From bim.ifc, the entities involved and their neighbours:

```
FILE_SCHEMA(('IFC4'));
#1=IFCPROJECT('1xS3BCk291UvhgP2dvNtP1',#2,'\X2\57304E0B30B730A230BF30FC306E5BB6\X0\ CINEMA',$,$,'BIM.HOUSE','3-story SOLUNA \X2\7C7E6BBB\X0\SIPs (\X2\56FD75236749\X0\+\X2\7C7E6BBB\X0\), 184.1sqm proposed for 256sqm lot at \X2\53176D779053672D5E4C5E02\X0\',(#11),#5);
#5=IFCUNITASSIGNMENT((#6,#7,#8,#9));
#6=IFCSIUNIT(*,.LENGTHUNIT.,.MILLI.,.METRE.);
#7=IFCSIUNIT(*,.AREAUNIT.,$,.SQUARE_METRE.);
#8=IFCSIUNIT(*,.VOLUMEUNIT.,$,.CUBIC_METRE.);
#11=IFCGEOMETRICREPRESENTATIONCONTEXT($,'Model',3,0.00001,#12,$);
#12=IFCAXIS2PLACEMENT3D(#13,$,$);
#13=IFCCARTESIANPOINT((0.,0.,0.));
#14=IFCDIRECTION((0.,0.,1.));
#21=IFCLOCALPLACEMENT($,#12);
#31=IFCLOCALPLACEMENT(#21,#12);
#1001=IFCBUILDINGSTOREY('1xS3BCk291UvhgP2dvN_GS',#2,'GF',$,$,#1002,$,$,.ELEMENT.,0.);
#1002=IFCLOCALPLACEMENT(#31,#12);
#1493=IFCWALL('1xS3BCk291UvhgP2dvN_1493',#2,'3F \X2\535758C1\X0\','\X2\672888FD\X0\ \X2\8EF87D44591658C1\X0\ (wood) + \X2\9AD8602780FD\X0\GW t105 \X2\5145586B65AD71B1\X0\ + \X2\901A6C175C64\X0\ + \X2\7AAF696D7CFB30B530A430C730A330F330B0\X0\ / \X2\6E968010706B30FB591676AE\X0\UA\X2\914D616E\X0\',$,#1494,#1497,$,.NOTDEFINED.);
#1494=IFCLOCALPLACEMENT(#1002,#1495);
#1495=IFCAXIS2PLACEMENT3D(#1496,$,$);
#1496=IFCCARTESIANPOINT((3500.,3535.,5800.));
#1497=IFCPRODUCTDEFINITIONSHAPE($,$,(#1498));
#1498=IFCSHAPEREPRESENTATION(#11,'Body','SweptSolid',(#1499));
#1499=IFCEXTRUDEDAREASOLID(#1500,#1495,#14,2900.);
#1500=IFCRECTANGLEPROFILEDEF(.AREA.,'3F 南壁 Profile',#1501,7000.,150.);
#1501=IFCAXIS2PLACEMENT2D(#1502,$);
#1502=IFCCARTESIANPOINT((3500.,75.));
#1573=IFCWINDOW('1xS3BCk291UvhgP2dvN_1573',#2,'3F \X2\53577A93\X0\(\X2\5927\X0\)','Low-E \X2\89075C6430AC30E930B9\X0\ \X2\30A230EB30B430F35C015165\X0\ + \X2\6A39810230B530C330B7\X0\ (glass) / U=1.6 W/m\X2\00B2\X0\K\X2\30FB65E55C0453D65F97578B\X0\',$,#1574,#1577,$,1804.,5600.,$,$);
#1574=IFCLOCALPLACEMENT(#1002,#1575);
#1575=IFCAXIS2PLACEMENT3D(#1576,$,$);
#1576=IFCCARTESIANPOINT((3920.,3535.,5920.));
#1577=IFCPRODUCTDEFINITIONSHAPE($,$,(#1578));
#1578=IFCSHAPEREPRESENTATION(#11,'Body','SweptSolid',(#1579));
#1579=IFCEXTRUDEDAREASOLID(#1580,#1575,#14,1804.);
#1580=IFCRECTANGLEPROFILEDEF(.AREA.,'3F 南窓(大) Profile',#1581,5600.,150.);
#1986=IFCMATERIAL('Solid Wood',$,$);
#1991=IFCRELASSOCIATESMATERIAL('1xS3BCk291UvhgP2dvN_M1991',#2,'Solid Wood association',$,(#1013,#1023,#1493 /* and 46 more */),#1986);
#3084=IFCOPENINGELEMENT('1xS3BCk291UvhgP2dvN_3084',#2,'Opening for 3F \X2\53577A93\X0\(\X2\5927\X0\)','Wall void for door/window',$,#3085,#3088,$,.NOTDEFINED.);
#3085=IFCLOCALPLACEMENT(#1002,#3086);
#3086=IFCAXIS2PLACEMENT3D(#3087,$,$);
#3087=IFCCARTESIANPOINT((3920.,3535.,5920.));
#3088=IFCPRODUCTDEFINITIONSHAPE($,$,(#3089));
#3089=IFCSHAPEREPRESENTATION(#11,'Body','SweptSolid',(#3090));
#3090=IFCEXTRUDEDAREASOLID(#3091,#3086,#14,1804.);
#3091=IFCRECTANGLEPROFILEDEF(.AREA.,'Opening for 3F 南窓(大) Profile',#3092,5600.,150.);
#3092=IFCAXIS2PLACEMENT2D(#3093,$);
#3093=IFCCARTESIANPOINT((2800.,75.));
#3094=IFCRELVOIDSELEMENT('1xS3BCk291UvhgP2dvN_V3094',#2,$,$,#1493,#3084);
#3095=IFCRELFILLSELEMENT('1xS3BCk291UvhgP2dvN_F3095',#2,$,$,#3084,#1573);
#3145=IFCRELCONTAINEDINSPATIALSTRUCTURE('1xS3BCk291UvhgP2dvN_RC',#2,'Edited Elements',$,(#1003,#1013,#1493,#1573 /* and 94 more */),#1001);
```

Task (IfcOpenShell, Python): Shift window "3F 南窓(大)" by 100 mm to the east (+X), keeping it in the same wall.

```python
import ifcopenshell
import ifcopenshell.api.geometry
import ifcopenshell.util.placement
import ifcopenshell.util.unit

model = ifcopenshell.open("bim.ifc")
unit_scale = ifcopenshell.util.unit.calculate_unit_scale(model)

window = model.by_guid("1xS3BCk291UvhgP2dvN_1573")
opening = window.FillsVoids[0].RelatingOpeningElement
wall = opening.VoidsElements[0].RelatingBuildingElement

wall_matrix = ifcopenshell.util.placement.get_local_placement(wall.ObjectPlacement)
shift = wall_matrix[:3, 0] * 0.1 / unit_scale
before = ifcopenshell.util.placement.get_local_placement(window.ObjectPlacement)[:3, 3].copy()

# The window is not placed relative to its opening, so move both.
for product in (opening, window):
    matrix = ifcopenshell.util.placement.get_local_placement(product.ObjectPlacement)
    matrix[:3, 3] += shift
    ifcopenshell.api.geometry.edit_object_placement(model, product=product, matrix=matrix, is_si=False)

after = ifcopenshell.util.placement.get_local_placement(window.ObjectPlacement)[:3, 3]
print("window moved by", (after - before).round(3) + 0.0)

model.write("bim_updated.ifc")
```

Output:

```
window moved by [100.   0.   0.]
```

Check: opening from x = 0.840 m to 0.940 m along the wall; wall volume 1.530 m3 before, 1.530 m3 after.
